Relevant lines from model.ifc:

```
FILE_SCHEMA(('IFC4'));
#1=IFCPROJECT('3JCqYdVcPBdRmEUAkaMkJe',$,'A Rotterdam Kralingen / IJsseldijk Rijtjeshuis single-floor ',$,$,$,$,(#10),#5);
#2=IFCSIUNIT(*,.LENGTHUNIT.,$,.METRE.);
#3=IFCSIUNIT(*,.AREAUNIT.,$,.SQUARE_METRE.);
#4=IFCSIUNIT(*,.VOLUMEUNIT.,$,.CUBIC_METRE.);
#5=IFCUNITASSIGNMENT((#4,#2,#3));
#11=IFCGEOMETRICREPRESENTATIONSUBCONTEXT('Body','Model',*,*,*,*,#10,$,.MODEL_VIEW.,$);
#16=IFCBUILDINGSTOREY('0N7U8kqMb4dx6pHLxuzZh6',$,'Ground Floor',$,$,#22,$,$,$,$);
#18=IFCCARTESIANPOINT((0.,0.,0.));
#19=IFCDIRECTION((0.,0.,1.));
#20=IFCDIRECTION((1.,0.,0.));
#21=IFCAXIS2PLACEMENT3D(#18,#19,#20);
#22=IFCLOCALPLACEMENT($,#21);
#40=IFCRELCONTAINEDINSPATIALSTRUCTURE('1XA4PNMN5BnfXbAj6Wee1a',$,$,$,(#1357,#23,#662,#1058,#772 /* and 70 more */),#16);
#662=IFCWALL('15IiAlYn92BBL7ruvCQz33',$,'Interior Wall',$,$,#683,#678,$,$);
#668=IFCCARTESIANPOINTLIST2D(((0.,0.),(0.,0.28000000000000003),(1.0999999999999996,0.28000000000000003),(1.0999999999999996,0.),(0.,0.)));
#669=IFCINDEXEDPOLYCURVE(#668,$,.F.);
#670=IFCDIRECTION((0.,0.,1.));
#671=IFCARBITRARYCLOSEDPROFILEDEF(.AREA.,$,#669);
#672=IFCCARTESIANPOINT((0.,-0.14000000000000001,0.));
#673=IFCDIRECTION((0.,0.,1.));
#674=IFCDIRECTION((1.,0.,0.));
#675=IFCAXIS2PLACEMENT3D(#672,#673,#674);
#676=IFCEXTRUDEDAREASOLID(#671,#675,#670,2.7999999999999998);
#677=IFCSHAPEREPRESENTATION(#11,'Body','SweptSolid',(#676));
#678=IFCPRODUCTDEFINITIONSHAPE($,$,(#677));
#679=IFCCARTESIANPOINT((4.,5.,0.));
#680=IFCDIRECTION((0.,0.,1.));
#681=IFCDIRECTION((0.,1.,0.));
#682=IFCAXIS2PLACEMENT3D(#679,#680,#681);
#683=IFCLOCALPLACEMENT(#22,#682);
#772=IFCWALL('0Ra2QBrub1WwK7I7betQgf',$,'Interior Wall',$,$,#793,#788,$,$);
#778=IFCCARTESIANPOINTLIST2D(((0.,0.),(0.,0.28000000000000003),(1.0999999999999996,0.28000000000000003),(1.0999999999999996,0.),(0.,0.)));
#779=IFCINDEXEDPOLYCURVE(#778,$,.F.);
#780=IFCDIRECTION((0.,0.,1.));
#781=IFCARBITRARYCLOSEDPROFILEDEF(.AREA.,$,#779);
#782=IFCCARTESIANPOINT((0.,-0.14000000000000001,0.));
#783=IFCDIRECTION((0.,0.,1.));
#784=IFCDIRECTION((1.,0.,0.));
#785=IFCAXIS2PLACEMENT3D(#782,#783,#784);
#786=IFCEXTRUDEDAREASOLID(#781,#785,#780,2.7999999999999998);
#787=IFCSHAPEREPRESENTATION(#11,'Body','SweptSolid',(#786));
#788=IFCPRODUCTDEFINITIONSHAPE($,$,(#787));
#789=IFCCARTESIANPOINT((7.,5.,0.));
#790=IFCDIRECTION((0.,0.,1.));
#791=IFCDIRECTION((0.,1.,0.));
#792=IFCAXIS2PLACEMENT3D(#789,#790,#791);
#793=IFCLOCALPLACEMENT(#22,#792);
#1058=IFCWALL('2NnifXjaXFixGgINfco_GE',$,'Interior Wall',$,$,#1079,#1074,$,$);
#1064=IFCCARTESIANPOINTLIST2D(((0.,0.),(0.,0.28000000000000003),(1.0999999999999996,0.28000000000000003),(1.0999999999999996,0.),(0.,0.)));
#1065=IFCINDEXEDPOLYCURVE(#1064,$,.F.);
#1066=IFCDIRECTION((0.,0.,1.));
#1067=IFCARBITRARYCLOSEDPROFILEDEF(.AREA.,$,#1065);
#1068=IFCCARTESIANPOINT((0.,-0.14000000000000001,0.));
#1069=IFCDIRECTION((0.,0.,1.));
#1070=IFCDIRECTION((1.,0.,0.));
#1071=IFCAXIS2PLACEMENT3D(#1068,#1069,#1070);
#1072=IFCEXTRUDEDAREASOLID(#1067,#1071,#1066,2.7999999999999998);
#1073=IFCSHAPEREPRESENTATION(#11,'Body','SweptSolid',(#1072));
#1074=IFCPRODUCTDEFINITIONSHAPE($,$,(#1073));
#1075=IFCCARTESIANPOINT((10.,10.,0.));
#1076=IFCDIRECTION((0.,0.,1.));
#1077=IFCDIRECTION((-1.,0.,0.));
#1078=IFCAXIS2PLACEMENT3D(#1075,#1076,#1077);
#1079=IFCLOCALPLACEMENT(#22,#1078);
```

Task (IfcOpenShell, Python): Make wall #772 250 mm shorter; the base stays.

```python
import ifcopenshell
import ifcopenshell.geom
import ifcopenshell.util.representation
import ifcopenshell.util.shape
import ifcopenshell.util.unit

model = ifcopenshell.open("model.ifc")
unit_scale = ifcopenshell.util.unit.calculate_unit_scale(model)
settings = ifcopenshell.geom.settings()


def volume(element):
    """Net volume in cubic metres, openings subtracted."""
    shape = ifcopenshell.geom.create_shape(settings, element)
    return ifcopenshell.util.shape.get_volume(shape.geometry)


wall = model.by_guid("0Ra2QBrub1WwK7I7betQgf")
before = volume(wall)

body = ifcopenshell.util.representation.get_representation(wall, "Model", "Body")
solid = body.Items[0]
old_height = solid.Depth
solid.Depth -= 0.25 / unit_scale
after = volume(wall)

print(f"height {old_height:g} -> {solid.Depth:g}, volume {before:.3f} -> {after:.3f} m3")

model.write("model-out.ifc")
```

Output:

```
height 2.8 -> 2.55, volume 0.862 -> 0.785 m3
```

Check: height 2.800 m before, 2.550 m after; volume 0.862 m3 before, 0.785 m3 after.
